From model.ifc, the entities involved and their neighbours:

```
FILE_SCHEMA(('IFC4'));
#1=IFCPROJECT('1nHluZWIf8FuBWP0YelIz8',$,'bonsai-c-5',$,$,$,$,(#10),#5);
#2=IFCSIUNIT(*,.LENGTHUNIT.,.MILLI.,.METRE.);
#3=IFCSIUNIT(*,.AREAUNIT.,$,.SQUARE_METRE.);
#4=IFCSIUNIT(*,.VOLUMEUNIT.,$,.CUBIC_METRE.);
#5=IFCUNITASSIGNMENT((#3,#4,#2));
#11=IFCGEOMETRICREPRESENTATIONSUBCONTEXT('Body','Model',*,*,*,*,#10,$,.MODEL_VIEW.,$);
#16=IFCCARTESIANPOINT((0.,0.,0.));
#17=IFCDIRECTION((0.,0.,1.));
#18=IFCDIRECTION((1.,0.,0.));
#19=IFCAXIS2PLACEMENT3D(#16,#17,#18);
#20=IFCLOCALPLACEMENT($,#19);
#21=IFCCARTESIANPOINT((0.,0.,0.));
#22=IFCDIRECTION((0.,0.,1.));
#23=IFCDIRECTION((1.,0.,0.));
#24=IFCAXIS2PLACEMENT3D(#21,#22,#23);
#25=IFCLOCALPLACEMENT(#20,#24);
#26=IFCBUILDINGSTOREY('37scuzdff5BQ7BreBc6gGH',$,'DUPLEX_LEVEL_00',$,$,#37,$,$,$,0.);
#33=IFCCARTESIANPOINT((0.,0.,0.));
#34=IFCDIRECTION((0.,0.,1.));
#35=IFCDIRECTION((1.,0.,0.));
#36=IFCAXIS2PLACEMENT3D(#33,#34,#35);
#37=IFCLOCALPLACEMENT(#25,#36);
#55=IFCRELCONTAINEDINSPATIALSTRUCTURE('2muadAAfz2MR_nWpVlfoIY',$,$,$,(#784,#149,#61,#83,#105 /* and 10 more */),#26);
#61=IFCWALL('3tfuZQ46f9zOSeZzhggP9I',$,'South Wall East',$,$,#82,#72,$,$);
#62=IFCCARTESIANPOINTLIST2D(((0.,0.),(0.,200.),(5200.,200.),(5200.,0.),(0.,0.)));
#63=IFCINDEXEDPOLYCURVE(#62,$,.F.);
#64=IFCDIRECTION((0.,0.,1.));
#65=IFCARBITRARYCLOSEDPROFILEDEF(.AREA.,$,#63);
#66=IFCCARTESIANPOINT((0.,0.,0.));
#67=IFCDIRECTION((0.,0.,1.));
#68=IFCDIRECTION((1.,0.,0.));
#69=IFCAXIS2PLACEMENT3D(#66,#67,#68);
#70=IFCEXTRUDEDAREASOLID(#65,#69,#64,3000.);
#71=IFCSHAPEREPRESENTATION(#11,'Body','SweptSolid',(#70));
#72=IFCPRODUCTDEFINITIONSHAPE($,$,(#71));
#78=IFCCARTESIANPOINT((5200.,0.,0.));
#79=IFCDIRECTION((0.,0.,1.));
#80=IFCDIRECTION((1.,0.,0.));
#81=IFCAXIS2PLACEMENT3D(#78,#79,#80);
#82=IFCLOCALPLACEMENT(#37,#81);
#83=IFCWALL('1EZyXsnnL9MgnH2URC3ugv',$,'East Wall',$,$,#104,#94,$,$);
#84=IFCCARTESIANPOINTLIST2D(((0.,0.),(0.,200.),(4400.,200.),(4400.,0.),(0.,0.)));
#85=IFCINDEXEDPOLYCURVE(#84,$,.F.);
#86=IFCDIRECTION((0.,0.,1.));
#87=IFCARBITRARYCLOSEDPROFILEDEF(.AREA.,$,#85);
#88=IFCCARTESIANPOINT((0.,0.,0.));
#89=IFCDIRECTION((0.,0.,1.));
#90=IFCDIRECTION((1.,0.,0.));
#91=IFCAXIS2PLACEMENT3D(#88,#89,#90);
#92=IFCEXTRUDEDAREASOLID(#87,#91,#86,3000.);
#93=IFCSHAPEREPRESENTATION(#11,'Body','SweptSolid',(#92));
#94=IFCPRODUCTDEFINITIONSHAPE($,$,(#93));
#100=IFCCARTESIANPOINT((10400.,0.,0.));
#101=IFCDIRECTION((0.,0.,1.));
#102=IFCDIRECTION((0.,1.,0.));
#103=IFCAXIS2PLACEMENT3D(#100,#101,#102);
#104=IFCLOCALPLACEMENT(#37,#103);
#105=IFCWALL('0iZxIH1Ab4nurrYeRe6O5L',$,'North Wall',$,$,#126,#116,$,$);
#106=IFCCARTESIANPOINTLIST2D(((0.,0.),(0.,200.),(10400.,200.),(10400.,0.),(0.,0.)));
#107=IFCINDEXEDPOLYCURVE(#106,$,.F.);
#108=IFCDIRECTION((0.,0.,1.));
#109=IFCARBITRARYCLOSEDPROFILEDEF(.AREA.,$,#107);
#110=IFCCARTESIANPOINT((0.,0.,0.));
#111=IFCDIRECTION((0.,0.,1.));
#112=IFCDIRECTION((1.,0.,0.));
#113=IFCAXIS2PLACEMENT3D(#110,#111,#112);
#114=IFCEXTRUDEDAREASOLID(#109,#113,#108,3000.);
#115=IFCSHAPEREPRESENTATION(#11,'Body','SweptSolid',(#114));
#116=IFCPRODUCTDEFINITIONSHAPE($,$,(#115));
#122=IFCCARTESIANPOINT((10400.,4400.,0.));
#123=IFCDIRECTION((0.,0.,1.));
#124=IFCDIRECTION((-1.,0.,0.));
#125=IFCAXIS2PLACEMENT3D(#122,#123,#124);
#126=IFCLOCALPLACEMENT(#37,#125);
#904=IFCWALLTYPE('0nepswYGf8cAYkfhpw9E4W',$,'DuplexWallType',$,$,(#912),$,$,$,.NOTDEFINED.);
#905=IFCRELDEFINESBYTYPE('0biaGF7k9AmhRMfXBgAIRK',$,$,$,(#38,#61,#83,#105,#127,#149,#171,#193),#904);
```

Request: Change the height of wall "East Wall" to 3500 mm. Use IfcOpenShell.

```python
import ifcopenshell
import ifcopenshell.geom
import ifcopenshell.util.representation
import ifcopenshell.util.shape

model = ifcopenshell.open("model.ifc")
settings = ifcopenshell.geom.settings()


def volume(element):
    """Net volume in cubic metres, openings subtracted."""
    shape = ifcopenshell.geom.create_shape(settings, element)
    return ifcopenshell.util.shape.get_volume(shape.geometry)


wall = model.by_guid("1EZyXsnnL9MgnH2URC3ugv")
before = volume(wall)

body = ifcopenshell.util.representation.get_representation(wall, "Model", "Body")
solid = body.Items[0]
old_height = solid.Depth
solid.Depth = 3500.0
after = volume(wall)

print(f"height {old_height:g} -> {solid.Depth:g}, volume {before:.3f} -> {after:.3f} m3")

model.write("model_rev.ifc")
```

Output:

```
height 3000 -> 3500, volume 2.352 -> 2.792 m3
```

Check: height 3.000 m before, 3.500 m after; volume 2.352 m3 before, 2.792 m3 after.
